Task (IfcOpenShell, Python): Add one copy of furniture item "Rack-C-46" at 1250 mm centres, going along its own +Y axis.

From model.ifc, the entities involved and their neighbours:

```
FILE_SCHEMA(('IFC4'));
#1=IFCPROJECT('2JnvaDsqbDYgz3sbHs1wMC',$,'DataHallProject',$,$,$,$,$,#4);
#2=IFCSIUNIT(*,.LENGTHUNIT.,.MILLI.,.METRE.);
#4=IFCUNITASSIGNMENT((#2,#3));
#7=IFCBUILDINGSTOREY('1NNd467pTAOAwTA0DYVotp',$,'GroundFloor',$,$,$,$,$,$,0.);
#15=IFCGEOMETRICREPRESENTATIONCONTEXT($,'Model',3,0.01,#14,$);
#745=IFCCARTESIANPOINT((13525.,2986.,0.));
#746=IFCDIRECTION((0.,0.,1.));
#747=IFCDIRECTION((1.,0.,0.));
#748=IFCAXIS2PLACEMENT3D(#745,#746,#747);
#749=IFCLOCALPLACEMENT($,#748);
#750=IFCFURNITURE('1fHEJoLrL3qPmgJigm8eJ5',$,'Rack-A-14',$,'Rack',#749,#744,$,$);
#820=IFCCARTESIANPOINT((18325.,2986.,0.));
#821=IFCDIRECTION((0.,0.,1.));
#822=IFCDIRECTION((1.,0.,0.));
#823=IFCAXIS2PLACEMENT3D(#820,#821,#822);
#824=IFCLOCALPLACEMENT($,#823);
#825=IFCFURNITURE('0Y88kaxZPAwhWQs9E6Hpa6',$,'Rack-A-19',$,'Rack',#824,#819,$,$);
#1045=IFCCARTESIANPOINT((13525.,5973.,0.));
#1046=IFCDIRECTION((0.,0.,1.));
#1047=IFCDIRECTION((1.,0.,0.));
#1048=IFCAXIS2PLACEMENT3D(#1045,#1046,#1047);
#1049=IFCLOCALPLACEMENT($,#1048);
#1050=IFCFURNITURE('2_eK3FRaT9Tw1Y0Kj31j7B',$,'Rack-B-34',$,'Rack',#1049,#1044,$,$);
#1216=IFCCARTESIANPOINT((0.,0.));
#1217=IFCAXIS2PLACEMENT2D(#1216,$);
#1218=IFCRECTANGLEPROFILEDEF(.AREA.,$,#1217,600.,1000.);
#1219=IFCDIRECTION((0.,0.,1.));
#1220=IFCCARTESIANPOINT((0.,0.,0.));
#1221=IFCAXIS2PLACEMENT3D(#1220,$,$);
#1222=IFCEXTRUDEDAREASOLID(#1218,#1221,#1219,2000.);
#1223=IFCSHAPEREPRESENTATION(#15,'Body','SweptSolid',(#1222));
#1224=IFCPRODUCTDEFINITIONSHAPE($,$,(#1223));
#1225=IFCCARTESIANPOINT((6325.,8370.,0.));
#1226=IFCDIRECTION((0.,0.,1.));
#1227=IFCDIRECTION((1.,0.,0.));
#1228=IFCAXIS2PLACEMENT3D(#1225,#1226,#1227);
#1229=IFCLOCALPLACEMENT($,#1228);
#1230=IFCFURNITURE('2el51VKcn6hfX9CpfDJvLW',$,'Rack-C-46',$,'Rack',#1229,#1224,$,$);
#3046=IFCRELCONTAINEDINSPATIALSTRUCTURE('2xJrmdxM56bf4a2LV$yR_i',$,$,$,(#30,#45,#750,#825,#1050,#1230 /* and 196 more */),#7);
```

```python
import ifcopenshell
import ifcopenshell.api.geometry
import ifcopenshell.api.root
import ifcopenshell.util.element
import ifcopenshell.util.placement

model = ifcopenshell.open("model.ifc")

source = model.by_guid("2el51VKcn6hfX9CpfDJvLW")
base = ifcopenshell.util.placement.get_local_placement(source.ObjectPlacement)
step = base[:3, 1] * 1250.0

for i in range(1, 2):
    copy = ifcopenshell.api.root.copy_class(model, product=source)
    copy.Representation = ifcopenshell.util.element.copy_deep(
        model, source.Representation, exclude=["IfcGeometricRepresentationContext", "IfcRepresentationMap"]
    )
    matrix = base.copy()
    matrix[:3, 3] += i * step
    print("added at", matrix[:3, 3].round(3) + 0.0)
    ifcopenshell.api.geometry.edit_object_placement(model, product=copy, matrix=matrix, is_si=False)

model.write("model_rev.ifc")
```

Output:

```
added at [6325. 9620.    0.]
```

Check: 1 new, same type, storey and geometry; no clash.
